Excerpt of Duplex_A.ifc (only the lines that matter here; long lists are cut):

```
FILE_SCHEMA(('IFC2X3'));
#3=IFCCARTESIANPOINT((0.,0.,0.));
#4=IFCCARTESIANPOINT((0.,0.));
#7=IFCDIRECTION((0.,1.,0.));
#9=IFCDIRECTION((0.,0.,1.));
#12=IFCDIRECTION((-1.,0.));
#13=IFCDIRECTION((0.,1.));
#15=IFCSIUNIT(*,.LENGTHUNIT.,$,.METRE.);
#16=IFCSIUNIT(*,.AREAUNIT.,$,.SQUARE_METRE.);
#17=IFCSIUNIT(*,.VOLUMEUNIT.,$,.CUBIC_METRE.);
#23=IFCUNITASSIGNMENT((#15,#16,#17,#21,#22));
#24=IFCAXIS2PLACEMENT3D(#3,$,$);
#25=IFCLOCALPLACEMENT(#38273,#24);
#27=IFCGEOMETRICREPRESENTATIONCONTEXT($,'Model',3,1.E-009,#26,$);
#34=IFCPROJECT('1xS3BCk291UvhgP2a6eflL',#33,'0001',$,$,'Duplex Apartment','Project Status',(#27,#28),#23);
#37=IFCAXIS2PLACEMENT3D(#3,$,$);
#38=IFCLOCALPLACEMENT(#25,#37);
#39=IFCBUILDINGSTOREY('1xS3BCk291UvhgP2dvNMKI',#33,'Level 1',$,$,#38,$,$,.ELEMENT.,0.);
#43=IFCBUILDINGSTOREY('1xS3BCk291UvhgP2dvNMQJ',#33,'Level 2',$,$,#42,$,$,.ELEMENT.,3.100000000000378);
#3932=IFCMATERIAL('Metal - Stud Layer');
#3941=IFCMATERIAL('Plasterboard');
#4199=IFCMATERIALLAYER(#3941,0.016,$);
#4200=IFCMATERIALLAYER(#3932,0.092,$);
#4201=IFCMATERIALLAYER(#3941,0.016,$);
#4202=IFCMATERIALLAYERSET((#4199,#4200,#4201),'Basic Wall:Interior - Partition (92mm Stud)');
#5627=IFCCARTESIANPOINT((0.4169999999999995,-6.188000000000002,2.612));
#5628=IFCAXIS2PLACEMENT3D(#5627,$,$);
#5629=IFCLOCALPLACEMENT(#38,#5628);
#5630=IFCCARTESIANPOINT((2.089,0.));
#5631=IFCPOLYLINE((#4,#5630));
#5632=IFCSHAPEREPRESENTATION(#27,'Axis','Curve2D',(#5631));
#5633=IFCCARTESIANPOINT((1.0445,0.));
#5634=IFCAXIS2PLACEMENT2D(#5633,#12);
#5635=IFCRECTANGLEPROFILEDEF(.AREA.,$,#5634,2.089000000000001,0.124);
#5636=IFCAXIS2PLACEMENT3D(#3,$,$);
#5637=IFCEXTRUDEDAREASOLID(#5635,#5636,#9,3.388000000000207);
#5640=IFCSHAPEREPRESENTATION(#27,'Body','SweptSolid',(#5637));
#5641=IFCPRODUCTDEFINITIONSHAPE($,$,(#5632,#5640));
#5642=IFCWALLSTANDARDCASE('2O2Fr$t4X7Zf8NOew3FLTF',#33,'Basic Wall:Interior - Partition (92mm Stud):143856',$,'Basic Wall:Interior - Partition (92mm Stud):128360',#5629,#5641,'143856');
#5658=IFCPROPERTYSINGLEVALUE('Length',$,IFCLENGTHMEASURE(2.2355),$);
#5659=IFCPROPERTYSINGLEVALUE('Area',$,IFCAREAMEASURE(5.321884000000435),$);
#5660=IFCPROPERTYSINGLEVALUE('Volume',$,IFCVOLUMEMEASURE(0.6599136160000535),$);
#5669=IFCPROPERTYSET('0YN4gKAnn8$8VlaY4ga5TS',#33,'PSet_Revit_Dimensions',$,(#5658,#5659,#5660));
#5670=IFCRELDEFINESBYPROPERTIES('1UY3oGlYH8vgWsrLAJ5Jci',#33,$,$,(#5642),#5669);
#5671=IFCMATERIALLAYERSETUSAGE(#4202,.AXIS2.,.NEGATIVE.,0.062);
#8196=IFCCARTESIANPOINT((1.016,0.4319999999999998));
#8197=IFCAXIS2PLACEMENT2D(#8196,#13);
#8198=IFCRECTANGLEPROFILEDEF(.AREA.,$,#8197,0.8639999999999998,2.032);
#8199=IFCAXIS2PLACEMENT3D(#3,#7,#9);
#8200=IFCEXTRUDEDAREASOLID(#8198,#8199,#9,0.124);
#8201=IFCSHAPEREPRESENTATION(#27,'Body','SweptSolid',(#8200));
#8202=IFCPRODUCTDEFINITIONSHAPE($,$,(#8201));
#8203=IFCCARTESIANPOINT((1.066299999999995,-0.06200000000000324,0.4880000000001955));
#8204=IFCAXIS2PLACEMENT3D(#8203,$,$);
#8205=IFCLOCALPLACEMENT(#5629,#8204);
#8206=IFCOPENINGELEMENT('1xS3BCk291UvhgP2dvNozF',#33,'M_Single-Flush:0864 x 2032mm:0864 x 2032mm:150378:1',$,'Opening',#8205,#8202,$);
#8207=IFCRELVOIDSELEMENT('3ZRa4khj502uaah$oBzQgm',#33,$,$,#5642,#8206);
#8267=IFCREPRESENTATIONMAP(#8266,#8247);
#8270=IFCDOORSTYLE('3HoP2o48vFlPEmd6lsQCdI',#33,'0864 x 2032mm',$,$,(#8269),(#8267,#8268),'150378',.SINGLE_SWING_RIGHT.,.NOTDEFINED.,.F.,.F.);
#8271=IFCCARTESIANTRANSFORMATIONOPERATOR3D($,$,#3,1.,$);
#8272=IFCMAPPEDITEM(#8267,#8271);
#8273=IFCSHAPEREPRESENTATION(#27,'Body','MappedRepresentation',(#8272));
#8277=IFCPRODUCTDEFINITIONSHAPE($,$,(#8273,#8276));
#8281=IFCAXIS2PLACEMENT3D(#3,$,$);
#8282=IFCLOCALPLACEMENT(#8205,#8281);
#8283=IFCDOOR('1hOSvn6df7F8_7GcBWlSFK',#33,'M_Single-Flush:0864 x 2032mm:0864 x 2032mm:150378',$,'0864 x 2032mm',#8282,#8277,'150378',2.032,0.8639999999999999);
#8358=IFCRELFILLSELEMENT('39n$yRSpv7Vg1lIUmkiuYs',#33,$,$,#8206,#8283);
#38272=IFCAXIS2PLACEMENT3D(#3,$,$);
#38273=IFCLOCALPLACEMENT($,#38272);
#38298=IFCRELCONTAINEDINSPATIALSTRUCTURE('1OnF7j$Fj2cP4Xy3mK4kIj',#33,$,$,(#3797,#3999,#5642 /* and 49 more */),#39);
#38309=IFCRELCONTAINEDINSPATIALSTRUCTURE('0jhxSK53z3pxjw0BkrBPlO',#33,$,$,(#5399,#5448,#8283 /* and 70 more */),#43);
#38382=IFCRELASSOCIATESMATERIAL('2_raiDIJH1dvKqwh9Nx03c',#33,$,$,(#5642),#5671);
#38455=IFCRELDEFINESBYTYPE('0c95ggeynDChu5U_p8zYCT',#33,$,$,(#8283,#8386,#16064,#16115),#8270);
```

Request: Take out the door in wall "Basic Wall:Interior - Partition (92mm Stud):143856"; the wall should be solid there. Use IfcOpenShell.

```python
import ifcopenshell
import ifcopenshell.api.feature
import ifcopenshell.api.pset
import ifcopenshell.api.root
import ifcopenshell.geom
import ifcopenshell.util.element
import ifcopenshell.util.shape
import ifcopenshell.util.unit

model = ifcopenshell.open("Duplex_A.ifc")
area_scale = ifcopenshell.util.unit.calculate_unit_scale(model, "AREAUNIT")
volume_scale = ifcopenshell.util.unit.calculate_unit_scale(model, "VOLUMEUNIT")
settings = ifcopenshell.geom.settings()


def volume(element):
    """Net volume in cubic metres, openings subtracted."""
    shape = ifcopenshell.geom.create_shape(settings, element)
    return ifcopenshell.util.shape.get_volume(shape.geometry)


door = model.by_id(8283)
opening = door.FillsVoids[0].RelatingOpeningElement
wall = opening.VoidsElements[0].RelatingBuildingElement
before = volume(wall)

ifcopenshell.api.root.remove_product(model, product=door)
ifcopenshell.api.feature.remove_feature(model, feature=opening)

after = volume(wall)
thickness = 0.124  # wall thickness in metres

# Update the wall's stored quantities.
pset = model.by_id(ifcopenshell.util.element.get_pset(wall, "PSet_Revit_Dimensions", should_inherit=False)["id"])
ifcopenshell.api.pset.edit_pset(model, pset=pset, properties={
    "Area": model.create_entity("IfcAreaMeasure", after / thickness / area_scale),
    "Volume": model.create_entity("IfcVolumeMeasure", after / volume_scale),
})

print(f"wall volume {before:.3f} -> {after:.3f} m3")

model.write("Duplex_A_v2.ifc")
```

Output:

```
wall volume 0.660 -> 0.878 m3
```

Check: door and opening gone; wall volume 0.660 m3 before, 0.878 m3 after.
